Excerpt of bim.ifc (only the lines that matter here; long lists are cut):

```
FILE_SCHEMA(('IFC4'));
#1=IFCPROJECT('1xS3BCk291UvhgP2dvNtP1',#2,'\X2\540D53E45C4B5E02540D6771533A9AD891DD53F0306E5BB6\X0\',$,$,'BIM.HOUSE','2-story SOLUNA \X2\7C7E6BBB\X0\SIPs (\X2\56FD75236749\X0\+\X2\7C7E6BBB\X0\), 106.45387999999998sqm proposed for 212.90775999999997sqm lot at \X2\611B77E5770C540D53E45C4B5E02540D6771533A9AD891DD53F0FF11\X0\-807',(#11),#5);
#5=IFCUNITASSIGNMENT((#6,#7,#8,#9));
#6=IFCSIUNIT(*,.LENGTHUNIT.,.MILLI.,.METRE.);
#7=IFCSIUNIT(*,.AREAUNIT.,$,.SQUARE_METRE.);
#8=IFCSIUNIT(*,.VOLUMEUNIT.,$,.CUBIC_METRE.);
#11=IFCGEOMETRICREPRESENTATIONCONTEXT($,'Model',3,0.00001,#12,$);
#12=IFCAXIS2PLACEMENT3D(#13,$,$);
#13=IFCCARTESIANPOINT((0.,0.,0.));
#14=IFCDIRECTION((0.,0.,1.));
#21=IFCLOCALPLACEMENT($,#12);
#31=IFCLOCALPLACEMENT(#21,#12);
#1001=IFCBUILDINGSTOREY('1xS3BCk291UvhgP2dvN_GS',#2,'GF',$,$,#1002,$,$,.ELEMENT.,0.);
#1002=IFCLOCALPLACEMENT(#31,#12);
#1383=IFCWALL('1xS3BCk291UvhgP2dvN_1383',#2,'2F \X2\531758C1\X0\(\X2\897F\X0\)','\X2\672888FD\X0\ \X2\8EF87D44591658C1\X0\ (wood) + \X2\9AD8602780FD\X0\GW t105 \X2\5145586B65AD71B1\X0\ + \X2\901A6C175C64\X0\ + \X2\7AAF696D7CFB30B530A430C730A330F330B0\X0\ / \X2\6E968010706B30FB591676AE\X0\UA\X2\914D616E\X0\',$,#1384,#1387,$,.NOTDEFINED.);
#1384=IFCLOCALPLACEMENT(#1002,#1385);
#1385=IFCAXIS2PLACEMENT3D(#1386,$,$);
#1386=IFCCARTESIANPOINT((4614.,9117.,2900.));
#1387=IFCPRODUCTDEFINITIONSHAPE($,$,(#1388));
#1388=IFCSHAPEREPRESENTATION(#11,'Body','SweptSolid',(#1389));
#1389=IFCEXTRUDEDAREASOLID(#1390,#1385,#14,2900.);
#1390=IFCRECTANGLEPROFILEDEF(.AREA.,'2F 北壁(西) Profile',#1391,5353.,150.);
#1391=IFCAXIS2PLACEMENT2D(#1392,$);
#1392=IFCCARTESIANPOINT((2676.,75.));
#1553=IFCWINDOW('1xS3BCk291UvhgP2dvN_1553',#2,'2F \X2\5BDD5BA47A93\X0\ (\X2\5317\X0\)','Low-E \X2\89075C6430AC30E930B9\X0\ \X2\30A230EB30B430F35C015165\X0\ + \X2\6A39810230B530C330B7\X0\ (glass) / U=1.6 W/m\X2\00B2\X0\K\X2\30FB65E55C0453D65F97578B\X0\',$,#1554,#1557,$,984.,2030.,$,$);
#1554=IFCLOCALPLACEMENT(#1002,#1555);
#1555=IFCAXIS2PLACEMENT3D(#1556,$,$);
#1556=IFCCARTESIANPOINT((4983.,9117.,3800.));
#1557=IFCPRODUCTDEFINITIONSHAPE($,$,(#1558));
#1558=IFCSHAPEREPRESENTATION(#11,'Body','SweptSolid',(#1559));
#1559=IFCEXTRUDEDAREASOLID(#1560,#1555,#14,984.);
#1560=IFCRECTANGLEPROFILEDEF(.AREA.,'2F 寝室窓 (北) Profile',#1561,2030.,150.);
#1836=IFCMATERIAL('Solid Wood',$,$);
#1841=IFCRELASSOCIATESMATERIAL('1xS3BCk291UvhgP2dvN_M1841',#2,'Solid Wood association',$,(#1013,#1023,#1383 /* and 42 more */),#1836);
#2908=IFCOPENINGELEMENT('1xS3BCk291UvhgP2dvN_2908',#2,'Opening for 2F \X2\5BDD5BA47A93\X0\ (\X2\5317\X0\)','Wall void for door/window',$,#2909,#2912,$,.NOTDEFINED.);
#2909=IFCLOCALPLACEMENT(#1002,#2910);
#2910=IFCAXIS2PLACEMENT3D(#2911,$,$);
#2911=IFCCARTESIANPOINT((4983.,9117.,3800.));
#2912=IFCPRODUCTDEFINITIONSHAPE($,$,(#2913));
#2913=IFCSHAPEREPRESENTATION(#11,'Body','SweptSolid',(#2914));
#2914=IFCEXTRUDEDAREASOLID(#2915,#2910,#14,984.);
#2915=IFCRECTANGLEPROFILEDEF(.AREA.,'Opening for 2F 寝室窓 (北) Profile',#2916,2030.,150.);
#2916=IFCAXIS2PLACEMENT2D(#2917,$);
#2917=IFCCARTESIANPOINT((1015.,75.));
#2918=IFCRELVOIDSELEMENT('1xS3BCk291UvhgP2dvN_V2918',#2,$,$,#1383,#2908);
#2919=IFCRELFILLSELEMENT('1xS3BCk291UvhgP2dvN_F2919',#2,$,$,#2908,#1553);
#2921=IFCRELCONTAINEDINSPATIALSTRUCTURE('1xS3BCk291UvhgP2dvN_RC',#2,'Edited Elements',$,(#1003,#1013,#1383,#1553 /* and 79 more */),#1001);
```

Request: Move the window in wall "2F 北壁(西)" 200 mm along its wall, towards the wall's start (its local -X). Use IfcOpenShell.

```python
import ifcopenshell
import ifcopenshell.api.geometry
import ifcopenshell.util.placement
import ifcopenshell.util.unit

model = ifcopenshell.open("bim.ifc")
unit_scale = ifcopenshell.util.unit.calculate_unit_scale(model)

window = model.by_id(1553)
opening = window.FillsVoids[0].RelatingOpeningElement
wall = opening.VoidsElements[0].RelatingBuildingElement

wall_matrix = ifcopenshell.util.placement.get_local_placement(wall.ObjectPlacement)
shift = wall_matrix[:3, 0] * -0.2 / unit_scale
before = ifcopenshell.util.placement.get_local_placement(window.ObjectPlacement)[:3, 3].copy()

# The window is not placed relative to its opening, so move both.
for product in (opening, window):
    matrix = ifcopenshell.util.placement.get_local_placement(product.ObjectPlacement)
    matrix[:3, 3] += shift
    ifcopenshell.api.geometry.edit_object_placement(model, product=product, matrix=matrix, is_si=False)

after = ifcopenshell.util.placement.get_local_placement(window.ObjectPlacement)[:3, 3]
print("window moved by", (after - before).round(3) + 0.0)

model.write("bim_edited.ifc")
```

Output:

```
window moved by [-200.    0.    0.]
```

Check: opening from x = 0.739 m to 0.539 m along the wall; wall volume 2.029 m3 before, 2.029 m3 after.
